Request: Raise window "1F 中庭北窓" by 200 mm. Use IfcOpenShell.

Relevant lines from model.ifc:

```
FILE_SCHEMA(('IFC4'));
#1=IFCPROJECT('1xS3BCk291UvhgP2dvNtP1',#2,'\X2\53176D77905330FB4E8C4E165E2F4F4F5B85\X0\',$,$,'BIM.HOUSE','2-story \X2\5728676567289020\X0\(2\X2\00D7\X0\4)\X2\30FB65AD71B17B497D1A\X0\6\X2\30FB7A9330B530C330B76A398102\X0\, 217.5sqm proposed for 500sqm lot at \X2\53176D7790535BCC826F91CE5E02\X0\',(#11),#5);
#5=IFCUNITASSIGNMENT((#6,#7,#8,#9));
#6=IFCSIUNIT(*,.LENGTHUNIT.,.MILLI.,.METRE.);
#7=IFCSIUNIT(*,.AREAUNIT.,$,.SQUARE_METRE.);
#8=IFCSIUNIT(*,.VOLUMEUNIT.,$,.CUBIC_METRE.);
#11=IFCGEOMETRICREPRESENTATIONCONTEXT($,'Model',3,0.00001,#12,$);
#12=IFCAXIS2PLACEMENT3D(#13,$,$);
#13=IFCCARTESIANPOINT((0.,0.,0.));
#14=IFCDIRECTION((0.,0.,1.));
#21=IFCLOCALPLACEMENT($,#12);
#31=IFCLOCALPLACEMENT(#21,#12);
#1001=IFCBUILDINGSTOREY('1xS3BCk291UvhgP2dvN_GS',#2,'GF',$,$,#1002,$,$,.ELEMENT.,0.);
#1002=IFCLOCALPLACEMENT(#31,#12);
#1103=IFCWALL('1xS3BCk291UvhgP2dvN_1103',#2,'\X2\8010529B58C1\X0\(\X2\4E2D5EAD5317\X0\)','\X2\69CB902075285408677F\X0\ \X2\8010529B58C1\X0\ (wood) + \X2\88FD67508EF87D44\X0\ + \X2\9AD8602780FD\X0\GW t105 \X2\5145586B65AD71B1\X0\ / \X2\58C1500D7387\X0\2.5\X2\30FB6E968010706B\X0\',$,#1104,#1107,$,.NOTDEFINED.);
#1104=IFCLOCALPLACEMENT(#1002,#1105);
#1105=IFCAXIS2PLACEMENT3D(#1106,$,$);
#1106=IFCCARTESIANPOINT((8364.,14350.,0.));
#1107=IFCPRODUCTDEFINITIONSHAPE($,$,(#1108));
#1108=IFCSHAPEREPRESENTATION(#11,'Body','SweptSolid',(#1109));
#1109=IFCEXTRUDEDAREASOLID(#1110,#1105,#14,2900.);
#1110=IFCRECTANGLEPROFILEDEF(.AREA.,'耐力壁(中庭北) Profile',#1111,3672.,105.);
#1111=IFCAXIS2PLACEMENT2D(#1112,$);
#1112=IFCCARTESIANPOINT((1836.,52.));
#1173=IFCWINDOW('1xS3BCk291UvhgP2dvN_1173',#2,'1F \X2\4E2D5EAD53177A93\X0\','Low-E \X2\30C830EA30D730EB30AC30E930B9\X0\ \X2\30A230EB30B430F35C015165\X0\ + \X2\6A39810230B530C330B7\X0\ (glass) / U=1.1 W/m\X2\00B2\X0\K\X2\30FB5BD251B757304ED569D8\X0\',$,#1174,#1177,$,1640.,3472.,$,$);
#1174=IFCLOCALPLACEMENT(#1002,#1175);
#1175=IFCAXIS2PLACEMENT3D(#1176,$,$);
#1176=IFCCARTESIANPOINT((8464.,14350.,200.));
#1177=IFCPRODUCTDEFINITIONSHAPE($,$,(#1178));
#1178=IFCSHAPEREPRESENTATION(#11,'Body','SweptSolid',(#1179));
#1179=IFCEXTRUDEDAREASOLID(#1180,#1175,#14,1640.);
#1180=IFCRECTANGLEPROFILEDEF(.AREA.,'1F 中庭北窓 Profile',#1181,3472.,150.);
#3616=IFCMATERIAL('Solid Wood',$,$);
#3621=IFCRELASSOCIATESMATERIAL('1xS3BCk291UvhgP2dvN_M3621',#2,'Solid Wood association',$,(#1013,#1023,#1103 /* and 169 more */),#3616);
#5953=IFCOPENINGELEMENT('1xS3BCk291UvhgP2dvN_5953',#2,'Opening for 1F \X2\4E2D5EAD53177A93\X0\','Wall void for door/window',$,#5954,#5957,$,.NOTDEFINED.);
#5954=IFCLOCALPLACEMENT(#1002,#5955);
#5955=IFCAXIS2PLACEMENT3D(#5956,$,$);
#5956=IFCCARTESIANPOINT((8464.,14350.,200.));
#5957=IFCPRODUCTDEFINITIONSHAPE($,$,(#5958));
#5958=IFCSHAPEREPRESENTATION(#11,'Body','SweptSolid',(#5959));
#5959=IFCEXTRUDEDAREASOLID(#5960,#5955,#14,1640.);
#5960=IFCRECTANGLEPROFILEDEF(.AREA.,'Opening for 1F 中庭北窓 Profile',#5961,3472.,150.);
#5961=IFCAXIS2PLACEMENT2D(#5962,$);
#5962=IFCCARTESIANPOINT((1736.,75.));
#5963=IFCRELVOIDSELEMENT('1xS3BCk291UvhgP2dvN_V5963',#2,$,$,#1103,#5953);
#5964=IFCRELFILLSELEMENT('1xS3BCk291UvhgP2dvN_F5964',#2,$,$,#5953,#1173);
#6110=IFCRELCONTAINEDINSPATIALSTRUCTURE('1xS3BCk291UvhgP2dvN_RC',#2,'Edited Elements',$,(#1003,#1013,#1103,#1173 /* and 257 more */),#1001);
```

```python
import numpy as np
import ifcopenshell
import ifcopenshell.api.geometry
import ifcopenshell.util.placement
import ifcopenshell.util.unit

model = ifcopenshell.open("model.ifc")
unit_scale = ifcopenshell.util.unit.calculate_unit_scale(model)

window = model.by_id(1173)
opening = window.FillsVoids[0].RelatingOpeningElement
dz = 0.2 / unit_scale

shift = np.array([0.0, 0.0, dz])
# The window is not placed relative to its opening, so move both.
for product in (opening, window):
    matrix = ifcopenshell.util.placement.get_local_placement(product.ObjectPlacement)
    matrix[:3, 3] += shift
    ifcopenshell.api.geometry.edit_object_placement(model, product=product, matrix=matrix, is_si=False)

print(f"moved by {dz * unit_scale:+.3f} m")

model.write("model_updated.ifc")
```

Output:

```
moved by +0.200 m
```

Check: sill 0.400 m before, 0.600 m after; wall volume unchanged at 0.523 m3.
